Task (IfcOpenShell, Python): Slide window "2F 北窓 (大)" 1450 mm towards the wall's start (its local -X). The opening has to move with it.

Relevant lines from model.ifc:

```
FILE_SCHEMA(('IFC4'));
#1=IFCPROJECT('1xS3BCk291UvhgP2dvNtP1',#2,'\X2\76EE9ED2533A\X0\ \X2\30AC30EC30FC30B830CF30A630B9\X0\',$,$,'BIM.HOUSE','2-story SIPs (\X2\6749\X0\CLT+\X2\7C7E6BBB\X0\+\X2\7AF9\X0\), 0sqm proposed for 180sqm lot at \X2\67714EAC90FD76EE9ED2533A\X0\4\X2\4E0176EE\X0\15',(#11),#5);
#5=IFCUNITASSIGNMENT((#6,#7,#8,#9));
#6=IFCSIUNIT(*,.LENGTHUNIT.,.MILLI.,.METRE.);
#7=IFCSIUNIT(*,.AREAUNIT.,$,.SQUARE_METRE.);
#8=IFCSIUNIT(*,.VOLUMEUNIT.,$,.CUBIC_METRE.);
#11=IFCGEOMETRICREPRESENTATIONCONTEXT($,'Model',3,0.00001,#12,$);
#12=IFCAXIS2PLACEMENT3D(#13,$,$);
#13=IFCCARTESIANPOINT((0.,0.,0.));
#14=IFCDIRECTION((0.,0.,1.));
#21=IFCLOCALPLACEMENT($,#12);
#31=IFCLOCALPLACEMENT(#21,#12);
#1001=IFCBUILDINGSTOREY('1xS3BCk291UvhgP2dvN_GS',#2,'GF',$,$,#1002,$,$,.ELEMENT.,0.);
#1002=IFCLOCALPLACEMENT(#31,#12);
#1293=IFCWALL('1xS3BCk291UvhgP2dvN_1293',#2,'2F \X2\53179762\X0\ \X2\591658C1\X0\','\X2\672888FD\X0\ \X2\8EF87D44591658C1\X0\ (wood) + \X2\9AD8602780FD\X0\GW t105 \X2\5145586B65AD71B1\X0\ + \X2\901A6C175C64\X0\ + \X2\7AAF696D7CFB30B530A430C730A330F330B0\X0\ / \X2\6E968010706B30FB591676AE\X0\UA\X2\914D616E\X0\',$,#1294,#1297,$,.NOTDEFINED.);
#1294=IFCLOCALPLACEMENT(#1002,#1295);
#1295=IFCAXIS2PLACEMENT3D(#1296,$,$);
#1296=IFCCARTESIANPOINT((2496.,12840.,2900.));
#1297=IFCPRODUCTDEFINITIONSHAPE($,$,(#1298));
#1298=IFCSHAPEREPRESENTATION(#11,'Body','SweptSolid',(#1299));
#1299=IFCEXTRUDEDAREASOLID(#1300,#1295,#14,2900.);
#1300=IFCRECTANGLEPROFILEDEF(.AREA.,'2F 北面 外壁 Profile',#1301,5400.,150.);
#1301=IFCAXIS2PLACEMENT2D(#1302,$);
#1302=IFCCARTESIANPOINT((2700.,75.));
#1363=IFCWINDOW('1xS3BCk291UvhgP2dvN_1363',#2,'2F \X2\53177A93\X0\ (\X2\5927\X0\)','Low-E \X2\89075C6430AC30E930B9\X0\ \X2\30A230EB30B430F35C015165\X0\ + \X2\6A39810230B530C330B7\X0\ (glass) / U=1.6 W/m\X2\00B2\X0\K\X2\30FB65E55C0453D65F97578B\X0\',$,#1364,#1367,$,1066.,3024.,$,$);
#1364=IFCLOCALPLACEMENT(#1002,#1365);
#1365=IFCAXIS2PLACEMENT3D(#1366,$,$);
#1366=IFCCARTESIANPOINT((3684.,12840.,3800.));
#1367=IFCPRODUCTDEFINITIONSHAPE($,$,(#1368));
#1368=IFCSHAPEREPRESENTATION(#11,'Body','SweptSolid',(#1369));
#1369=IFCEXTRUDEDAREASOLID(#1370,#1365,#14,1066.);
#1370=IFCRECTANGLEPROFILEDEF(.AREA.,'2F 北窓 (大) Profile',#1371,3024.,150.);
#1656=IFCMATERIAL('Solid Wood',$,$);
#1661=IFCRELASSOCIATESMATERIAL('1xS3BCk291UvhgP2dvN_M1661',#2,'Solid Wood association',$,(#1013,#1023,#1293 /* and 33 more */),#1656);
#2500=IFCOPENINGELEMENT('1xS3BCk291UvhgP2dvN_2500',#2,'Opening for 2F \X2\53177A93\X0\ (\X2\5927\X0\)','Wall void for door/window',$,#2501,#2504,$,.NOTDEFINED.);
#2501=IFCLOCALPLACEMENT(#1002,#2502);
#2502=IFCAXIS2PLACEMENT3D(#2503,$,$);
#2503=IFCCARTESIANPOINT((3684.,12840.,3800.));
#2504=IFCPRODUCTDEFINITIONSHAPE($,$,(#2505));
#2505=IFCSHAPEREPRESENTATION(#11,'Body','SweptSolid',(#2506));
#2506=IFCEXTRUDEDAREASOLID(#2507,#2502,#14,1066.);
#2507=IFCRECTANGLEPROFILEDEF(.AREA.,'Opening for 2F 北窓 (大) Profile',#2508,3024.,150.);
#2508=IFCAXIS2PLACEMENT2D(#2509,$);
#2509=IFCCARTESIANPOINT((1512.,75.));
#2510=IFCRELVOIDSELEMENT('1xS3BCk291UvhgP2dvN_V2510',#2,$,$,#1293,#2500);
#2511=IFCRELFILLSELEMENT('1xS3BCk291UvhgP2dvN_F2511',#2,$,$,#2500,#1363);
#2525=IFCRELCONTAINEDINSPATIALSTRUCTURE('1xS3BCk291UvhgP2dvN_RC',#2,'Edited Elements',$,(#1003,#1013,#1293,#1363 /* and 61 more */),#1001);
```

```python
import ifcopenshell
import ifcopenshell.api.geometry
import ifcopenshell.util.placement
import ifcopenshell.util.unit

model = ifcopenshell.open("model.ifc")
unit_scale = ifcopenshell.util.unit.calculate_unit_scale(model)

window = model.by_id(1363)
opening = window.FillsVoids[0].RelatingOpeningElement
wall = opening.VoidsElements[0].RelatingBuildingElement

wall_matrix = ifcopenshell.util.placement.get_local_placement(wall.ObjectPlacement)
shift = wall_matrix[:3, 0] * -1.45 / unit_scale
before = ifcopenshell.util.placement.get_local_placement(window.ObjectPlacement)[:3, 3].copy()

# The window is not placed relative to its opening, so move both.
for product in (opening, window):
    matrix = ifcopenshell.util.placement.get_local_placement(product.ObjectPlacement)
    matrix[:3, 3] += shift
    ifcopenshell.api.geometry.edit_object_placement(model, product=product, matrix=matrix, is_si=False)

after = ifcopenshell.util.placement.get_local_placement(window.ObjectPlacement)[:3, 3]
print("window moved by", (after - before).round(3) + 0.0)

model.write("model_updated.ifc")
```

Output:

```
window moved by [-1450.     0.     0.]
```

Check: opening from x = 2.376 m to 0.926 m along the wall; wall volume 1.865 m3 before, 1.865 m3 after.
